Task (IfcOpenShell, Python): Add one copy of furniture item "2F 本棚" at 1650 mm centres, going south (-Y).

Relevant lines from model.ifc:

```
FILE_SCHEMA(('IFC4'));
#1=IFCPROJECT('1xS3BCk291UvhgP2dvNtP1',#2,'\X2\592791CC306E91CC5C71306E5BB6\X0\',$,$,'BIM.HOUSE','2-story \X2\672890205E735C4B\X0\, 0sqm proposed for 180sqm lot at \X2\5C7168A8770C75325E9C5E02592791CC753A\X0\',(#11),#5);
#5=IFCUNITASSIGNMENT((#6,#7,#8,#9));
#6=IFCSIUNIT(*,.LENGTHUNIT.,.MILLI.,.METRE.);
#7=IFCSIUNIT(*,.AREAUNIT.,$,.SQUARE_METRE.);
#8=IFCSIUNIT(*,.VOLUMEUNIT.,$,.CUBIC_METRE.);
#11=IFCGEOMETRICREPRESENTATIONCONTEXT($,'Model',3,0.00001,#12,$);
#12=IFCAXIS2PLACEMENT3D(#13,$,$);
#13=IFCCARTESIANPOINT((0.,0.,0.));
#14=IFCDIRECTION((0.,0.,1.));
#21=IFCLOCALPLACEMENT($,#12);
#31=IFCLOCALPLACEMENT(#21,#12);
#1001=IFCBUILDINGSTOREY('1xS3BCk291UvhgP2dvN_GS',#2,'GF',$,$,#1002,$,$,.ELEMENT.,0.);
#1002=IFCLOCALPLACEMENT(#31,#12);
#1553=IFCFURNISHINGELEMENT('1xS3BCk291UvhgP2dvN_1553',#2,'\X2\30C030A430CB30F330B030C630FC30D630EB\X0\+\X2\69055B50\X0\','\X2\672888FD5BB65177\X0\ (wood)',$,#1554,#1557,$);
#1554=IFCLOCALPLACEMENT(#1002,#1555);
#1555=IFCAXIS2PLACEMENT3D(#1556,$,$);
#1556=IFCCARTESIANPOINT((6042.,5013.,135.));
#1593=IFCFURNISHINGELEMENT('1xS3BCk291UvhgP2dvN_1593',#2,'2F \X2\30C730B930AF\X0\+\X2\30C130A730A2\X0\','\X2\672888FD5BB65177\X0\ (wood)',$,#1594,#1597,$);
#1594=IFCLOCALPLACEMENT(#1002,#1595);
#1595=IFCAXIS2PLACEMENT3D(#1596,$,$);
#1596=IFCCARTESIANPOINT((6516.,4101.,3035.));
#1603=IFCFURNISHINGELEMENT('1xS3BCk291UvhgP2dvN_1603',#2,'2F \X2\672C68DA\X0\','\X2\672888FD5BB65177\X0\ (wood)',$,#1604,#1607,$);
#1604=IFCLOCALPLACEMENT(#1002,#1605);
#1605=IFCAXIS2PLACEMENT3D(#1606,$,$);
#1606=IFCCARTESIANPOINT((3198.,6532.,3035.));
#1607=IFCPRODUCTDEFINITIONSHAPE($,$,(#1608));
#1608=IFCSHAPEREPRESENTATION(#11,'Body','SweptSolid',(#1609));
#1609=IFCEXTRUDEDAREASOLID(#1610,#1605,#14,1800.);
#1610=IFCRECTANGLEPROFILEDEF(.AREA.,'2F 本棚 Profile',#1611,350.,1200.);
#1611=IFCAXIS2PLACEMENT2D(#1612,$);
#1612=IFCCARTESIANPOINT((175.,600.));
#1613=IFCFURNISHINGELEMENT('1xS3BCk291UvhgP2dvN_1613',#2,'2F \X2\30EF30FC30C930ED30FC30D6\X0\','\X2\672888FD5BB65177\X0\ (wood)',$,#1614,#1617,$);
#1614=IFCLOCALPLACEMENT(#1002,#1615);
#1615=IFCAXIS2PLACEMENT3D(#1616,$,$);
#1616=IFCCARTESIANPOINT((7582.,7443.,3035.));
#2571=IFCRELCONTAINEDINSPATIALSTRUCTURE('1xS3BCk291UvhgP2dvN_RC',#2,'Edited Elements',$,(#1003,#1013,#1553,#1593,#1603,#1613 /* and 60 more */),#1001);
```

```python
import numpy as np
import ifcopenshell
import ifcopenshell.api.geometry
import ifcopenshell.api.root
import ifcopenshell.util.element
import ifcopenshell.util.placement

model = ifcopenshell.open("model.ifc")


def reuse_history(source, copy):
    """copy_class also copies each property set's owner history, people and application; keep the originals."""
    for rel in copy.IsDefinedBy:
        if rel.is_a("IfcRelDefinesByProperties") and (history := rel.RelatingPropertyDefinition.OwnerHistory):
            rel.RelatingPropertyDefinition.OwnerHistory = source.OwnerHistory
            ifcopenshell.util.element.remove_deep2(model, history)


source = model.by_id(1603)
base = ifcopenshell.util.placement.get_local_placement(source.ObjectPlacement)
step = np.array([0.0, -1.0, 0.0]) * 1650.0

for i in range(1, 2):
    copy = ifcopenshell.api.root.copy_class(model, product=source)
    copy.Representation = ifcopenshell.util.element.copy_deep(
        model, source.Representation, exclude=["IfcGeometricRepresentationContext", "IfcRepresentationMap"]
    )
    reuse_history(source, copy)
    matrix = base.copy()
    matrix[:3, 3] += i * step
    print("added at", matrix[:3, 3].round(3) + 0.0)
    ifcopenshell.api.geometry.edit_object_placement(model, product=copy, matrix=matrix, is_si=False)

model.write("model_rev.ifc")
```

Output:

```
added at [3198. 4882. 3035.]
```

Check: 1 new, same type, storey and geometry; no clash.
